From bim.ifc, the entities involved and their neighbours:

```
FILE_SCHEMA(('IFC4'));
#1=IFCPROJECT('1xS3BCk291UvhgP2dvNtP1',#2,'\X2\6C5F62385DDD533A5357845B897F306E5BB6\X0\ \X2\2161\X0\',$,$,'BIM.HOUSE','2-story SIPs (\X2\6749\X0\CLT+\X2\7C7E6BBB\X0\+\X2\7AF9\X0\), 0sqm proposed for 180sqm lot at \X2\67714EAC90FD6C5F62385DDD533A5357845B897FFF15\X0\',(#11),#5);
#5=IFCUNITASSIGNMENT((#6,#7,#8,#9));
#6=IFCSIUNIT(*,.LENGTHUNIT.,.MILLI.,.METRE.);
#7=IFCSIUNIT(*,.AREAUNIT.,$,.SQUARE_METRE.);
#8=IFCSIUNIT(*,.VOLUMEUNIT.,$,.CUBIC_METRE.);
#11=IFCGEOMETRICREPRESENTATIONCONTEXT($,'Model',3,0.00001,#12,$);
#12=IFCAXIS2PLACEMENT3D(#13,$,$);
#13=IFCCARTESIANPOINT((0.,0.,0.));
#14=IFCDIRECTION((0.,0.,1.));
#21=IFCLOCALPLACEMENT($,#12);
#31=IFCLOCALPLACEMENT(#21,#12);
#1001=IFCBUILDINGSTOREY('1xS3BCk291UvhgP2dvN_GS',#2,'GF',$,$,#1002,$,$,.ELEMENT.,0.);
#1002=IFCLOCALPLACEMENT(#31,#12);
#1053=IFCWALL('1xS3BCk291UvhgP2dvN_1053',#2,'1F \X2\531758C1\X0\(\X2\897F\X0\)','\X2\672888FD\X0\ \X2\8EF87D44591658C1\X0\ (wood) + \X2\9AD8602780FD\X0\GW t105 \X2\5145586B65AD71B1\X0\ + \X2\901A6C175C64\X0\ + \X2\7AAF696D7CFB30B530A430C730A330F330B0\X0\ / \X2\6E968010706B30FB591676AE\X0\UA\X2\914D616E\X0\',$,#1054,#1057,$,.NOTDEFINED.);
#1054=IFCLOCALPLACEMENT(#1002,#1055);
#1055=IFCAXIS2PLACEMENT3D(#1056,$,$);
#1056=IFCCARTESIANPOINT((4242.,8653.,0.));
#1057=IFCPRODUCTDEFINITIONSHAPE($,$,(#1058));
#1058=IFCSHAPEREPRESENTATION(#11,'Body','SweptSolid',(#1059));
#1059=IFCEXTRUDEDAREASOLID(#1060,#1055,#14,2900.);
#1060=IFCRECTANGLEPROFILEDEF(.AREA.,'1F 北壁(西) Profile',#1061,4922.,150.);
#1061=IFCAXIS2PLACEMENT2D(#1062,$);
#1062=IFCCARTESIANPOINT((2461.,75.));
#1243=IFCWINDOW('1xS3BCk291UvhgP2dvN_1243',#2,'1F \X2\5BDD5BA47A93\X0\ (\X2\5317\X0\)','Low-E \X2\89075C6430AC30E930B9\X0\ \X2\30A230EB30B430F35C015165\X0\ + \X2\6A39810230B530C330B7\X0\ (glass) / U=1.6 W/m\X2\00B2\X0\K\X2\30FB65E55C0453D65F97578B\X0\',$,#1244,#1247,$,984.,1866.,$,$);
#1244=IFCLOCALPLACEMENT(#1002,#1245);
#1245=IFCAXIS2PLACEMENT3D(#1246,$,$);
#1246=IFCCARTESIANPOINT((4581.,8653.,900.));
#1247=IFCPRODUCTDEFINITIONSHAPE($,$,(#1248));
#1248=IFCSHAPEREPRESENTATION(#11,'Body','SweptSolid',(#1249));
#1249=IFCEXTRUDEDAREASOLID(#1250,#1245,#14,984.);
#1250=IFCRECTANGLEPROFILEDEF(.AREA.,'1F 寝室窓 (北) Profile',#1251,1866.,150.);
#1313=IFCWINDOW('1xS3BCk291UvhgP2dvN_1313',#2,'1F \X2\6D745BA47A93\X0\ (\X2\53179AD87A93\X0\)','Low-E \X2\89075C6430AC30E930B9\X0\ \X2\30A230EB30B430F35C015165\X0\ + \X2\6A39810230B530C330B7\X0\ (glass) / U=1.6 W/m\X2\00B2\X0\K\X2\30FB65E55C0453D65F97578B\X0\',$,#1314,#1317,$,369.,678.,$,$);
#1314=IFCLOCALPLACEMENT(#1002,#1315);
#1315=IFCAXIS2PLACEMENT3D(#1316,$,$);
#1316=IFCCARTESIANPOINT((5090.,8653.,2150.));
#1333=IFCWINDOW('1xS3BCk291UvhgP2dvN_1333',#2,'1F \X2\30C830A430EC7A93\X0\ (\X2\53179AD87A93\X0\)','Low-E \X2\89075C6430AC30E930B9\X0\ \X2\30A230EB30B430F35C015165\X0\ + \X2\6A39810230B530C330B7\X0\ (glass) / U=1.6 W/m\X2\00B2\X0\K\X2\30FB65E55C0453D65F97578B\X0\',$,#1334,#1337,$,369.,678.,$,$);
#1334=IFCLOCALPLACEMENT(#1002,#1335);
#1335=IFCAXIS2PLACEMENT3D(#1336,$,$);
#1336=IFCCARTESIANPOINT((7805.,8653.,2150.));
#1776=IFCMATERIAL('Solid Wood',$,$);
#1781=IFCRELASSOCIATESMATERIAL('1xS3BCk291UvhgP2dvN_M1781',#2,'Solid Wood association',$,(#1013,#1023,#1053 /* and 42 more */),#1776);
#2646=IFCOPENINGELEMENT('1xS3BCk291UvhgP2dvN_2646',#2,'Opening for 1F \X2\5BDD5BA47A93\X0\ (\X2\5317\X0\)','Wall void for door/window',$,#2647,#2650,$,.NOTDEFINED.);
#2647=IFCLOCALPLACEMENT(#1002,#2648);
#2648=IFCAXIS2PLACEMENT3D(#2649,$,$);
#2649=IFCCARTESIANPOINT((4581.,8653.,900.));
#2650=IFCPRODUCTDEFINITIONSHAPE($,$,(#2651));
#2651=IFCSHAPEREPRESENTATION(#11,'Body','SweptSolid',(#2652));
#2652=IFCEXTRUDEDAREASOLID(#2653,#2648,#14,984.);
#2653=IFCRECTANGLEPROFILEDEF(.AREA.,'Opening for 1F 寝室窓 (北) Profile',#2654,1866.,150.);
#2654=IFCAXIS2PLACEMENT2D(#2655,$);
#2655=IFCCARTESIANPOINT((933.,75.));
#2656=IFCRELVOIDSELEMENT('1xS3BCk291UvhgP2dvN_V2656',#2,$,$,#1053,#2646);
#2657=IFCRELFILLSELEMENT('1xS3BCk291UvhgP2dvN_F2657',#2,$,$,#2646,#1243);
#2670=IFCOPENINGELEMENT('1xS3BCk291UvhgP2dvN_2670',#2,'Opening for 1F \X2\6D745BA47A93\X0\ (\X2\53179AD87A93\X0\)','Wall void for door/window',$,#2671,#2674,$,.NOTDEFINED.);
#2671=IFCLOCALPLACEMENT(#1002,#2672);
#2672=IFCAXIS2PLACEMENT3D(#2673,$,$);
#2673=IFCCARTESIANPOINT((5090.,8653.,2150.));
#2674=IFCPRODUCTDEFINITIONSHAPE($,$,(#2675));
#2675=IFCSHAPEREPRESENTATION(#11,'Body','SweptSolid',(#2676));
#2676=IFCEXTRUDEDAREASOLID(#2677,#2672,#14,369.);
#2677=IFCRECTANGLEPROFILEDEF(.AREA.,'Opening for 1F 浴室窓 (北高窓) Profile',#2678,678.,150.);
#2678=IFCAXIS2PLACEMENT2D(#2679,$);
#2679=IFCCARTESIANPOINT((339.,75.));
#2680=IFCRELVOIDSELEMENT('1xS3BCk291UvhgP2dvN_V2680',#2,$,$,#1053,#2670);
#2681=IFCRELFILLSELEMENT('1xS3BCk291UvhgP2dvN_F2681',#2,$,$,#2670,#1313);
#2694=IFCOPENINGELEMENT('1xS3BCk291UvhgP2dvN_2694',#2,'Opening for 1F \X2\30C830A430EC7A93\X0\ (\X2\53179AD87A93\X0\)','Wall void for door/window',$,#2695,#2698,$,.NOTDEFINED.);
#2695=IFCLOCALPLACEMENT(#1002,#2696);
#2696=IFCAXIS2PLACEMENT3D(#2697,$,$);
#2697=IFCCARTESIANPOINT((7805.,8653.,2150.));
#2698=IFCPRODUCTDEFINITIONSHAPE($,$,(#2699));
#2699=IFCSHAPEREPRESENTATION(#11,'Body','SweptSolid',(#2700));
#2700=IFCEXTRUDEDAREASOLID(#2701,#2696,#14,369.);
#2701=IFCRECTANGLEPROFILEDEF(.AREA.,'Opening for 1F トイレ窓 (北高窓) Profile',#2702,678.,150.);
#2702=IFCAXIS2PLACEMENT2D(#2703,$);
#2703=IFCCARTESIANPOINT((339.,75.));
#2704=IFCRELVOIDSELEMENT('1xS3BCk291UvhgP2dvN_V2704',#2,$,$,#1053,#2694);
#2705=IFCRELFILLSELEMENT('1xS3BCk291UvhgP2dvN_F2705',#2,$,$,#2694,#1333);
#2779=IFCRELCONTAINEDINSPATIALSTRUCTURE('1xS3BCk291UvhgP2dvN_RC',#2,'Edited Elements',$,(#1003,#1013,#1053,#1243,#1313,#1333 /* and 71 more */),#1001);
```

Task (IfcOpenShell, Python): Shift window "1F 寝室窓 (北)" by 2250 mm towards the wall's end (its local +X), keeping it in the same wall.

```python
import ifcopenshell
import ifcopenshell.api.geometry
import ifcopenshell.util.placement

model = ifcopenshell.open("bim.ifc")

window = model.by_guid("1xS3BCk291UvhgP2dvN_1243")
opening = window.FillsVoids[0].RelatingOpeningElement
wall = opening.VoidsElements[0].RelatingBuildingElement

wall_matrix = ifcopenshell.util.placement.get_local_placement(wall.ObjectPlacement)
shift = wall_matrix[:3, 0] * 2250.0
before = ifcopenshell.util.placement.get_local_placement(window.ObjectPlacement)[:3, 3].copy()

# The window is not placed relative to its opening, so move both.
for product in (opening, window):
    matrix = ifcopenshell.util.placement.get_local_placement(product.ObjectPlacement)
    matrix[:3, 3] += shift
    ifcopenshell.api.geometry.edit_object_placement(model, product=product, matrix=matrix, is_si=False)

after = ifcopenshell.util.placement.get_local_placement(window.ObjectPlacement)[:3, 3]
print("window moved by", (after - before).round(3) + 0.0)

model.write("bim_edited.ifc")
```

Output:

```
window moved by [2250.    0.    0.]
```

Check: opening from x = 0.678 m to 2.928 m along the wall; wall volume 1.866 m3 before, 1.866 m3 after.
